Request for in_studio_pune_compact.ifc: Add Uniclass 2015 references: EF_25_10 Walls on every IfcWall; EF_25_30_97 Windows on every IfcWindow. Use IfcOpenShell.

First a look at what the model holds.

```python
import ifcopenshell

model = ifcopenshell.open("in_studio_pune_compact.ifc")
print(model.schema)
print("classifications:", [c.Name for c in model.by_type("IfcClassification")])
for ifc_class in ("IfcDoor", "IfcRoof", "IfcStair", "IfcWall", "IfcWindow"):
    print(ifc_class, len(model.by_type(ifc_class)))
```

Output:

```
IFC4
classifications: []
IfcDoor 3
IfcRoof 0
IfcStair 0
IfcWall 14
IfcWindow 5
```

```python
import ifcopenshell
import ifcopenshell.api.classification

model = ifcopenshell.open("in_studio_pune_compact.ifc")

system = ifcopenshell.api.classification.add_classification(model, classification="Uniclass 2015")

codes = {
    "IfcWall": ("EF_25_10", "Walls"),
    "IfcWindow": ("EF_25_30_97", "Windows"),
}
for ifc_class, (code, name) in codes.items():
    products = model.by_type(ifc_class)
    ifcopenshell.api.classification.add_reference(
        model, products=products, classification=system, identification=code, name=name
    )
    print(code, len(products))

model.write("in_studio_pune_compact-out.ifc")
```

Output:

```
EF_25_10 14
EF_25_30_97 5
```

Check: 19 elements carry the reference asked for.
